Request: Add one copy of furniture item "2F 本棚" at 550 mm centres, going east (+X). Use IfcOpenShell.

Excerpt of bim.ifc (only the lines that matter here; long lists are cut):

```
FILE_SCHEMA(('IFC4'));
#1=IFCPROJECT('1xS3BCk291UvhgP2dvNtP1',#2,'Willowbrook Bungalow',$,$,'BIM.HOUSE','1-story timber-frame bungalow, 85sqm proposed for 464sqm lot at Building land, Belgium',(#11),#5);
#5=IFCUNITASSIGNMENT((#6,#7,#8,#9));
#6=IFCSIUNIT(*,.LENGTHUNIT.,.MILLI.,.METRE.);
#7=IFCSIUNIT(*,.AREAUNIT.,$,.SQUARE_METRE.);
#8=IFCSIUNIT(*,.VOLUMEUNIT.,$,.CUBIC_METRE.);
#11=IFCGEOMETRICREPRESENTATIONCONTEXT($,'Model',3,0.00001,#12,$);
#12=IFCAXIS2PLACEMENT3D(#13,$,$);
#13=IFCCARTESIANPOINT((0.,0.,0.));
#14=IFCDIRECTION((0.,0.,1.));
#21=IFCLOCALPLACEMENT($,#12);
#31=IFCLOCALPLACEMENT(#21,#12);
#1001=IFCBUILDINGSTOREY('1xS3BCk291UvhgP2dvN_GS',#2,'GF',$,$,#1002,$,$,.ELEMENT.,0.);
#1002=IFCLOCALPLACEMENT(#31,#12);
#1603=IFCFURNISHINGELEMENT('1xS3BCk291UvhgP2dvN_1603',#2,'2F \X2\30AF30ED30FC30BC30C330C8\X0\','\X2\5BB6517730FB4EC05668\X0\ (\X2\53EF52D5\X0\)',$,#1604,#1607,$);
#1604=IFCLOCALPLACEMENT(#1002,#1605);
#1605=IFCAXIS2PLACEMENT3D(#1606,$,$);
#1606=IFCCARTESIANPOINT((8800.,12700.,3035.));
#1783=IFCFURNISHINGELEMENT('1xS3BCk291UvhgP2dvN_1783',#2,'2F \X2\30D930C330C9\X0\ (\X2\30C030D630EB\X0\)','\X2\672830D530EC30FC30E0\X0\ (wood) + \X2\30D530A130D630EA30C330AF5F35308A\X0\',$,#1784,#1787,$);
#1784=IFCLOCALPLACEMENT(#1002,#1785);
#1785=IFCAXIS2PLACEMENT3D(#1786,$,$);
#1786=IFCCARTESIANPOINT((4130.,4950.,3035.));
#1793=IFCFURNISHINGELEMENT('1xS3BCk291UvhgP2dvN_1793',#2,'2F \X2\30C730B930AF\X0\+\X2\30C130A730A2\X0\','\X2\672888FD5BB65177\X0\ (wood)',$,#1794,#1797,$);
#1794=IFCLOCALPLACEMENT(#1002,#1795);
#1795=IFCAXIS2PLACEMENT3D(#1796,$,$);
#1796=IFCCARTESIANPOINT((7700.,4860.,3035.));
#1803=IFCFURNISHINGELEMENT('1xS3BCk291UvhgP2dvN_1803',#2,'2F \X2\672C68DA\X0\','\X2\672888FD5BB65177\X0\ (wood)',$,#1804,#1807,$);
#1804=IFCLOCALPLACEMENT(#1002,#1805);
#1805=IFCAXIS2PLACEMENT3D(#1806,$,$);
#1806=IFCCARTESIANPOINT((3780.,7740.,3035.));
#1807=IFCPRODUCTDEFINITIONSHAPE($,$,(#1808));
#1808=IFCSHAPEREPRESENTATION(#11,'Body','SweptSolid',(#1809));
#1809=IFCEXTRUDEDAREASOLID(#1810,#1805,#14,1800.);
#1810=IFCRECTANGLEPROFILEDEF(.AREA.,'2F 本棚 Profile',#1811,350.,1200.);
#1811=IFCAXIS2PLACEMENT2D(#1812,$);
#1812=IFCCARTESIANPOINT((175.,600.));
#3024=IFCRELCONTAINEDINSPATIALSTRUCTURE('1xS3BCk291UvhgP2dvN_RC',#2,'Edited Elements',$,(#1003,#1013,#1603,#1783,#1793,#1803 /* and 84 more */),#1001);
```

```python
import numpy as np
import ifcopenshell
import ifcopenshell.api.geometry
import ifcopenshell.api.root
import ifcopenshell.util.element
import ifcopenshell.util.placement
import ifcopenshell.util.unit

model = ifcopenshell.open("bim.ifc")
unit_scale = ifcopenshell.util.unit.calculate_unit_scale(model)


def reuse_history(source, copy):
    """copy_class also copies each property set's owner history, people and application; keep the originals."""
    for rel in copy.IsDefinedBy:
        if rel.is_a("IfcRelDefinesByProperties") and (history := rel.RelatingPropertyDefinition.OwnerHistory):
            rel.RelatingPropertyDefinition.OwnerHistory = source.OwnerHistory
            ifcopenshell.util.element.remove_deep2(model, history)


source = model.by_id(1803)
base = ifcopenshell.util.placement.get_local_placement(source.ObjectPlacement)
step = np.array([1.0, 0.0, 0.0]) * 0.55 / unit_scale

for i in range(1, 2):
    copy = ifcopenshell.api.root.copy_class(model, product=source)
    copy.Representation = ifcopenshell.util.element.copy_deep(
        model, source.Representation, exclude=["IfcGeometricRepresentationContext", "IfcRepresentationMap"]
    )
    reuse_history(source, copy)
    matrix = base.copy()
    matrix[:3, 3] += i * step
    print("added at", matrix[:3, 3].round(3) + 0.0)
    ifcopenshell.api.geometry.edit_object_placement(model, product=copy, matrix=matrix, is_si=False)

model.write("bim_edited.ifc")
```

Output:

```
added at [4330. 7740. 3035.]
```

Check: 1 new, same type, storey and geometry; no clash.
